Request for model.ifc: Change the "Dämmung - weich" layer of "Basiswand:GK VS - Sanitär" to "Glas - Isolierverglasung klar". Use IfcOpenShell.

First a look at what the model holds.

```python
import ifcopenshell
import ifcopenshell.util.element

model = ifcopenshell.open("model.ifc")
print(model.schema)
for layer_set in model.by_type("IfcMaterialLayerSet"):
    if layer_set.LayerSetName == "Basiswand:GK VS - Sanitär":
        for layer in layer_set.MaterialLayers:
            print(layer.id(), layer.Material and layer.Material.Name, layer.LayerThickness, sep=" | ")
        print(len(ifcopenshell.util.element.get_elements_by_material(model, layer_set)), "elements and types use it")
print(sorted(m.Name for m in model.by_type("IfcMaterial") if m.Name)[:60])
```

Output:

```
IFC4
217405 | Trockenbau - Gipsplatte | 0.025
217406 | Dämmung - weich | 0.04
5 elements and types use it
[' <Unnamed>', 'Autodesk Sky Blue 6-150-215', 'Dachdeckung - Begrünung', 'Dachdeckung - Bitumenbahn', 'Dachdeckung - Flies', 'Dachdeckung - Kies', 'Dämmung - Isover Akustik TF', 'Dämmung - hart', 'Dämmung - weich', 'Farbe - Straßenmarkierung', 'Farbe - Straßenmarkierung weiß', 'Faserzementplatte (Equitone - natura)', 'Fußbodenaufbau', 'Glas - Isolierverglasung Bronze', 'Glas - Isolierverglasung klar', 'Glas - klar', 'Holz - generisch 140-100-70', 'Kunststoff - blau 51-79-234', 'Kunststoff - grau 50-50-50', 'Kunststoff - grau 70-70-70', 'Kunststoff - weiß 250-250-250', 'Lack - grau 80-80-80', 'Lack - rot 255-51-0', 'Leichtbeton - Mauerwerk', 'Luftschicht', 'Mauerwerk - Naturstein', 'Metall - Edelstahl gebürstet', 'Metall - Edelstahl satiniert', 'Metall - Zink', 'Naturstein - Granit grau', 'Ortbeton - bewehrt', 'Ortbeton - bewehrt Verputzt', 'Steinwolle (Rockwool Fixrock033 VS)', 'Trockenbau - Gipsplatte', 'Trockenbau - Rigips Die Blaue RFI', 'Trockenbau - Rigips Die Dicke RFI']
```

```python
import ifcopenshell
import ifcopenshell.api.material

model = ifcopenshell.open("model.ifc")

layer_set = next(s for s in model.by_type("IfcMaterialLayerSet") if s.LayerSetName == "Basiswand:GK VS - Sanitär")
layer = next(l for l in layer_set.MaterialLayers if l.Material and l.Material.Name == "Dämmung - weich")
material = next(m for m in model.by_type("IfcMaterial") if m.Name == "Glas - Isolierverglasung klar")

# Point this one layer at the other material; renaming the old one would change it everywhere.
ifcopenshell.api.material.edit_layer(model, layer=layer, attributes={"Name": material.Name}, material=material)

print([l.Material.Name if l.Material else None for l in layer_set.MaterialLayers])

model.write("model_v2.ifc")
```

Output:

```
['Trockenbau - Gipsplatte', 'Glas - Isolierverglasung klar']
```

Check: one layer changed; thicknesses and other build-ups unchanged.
